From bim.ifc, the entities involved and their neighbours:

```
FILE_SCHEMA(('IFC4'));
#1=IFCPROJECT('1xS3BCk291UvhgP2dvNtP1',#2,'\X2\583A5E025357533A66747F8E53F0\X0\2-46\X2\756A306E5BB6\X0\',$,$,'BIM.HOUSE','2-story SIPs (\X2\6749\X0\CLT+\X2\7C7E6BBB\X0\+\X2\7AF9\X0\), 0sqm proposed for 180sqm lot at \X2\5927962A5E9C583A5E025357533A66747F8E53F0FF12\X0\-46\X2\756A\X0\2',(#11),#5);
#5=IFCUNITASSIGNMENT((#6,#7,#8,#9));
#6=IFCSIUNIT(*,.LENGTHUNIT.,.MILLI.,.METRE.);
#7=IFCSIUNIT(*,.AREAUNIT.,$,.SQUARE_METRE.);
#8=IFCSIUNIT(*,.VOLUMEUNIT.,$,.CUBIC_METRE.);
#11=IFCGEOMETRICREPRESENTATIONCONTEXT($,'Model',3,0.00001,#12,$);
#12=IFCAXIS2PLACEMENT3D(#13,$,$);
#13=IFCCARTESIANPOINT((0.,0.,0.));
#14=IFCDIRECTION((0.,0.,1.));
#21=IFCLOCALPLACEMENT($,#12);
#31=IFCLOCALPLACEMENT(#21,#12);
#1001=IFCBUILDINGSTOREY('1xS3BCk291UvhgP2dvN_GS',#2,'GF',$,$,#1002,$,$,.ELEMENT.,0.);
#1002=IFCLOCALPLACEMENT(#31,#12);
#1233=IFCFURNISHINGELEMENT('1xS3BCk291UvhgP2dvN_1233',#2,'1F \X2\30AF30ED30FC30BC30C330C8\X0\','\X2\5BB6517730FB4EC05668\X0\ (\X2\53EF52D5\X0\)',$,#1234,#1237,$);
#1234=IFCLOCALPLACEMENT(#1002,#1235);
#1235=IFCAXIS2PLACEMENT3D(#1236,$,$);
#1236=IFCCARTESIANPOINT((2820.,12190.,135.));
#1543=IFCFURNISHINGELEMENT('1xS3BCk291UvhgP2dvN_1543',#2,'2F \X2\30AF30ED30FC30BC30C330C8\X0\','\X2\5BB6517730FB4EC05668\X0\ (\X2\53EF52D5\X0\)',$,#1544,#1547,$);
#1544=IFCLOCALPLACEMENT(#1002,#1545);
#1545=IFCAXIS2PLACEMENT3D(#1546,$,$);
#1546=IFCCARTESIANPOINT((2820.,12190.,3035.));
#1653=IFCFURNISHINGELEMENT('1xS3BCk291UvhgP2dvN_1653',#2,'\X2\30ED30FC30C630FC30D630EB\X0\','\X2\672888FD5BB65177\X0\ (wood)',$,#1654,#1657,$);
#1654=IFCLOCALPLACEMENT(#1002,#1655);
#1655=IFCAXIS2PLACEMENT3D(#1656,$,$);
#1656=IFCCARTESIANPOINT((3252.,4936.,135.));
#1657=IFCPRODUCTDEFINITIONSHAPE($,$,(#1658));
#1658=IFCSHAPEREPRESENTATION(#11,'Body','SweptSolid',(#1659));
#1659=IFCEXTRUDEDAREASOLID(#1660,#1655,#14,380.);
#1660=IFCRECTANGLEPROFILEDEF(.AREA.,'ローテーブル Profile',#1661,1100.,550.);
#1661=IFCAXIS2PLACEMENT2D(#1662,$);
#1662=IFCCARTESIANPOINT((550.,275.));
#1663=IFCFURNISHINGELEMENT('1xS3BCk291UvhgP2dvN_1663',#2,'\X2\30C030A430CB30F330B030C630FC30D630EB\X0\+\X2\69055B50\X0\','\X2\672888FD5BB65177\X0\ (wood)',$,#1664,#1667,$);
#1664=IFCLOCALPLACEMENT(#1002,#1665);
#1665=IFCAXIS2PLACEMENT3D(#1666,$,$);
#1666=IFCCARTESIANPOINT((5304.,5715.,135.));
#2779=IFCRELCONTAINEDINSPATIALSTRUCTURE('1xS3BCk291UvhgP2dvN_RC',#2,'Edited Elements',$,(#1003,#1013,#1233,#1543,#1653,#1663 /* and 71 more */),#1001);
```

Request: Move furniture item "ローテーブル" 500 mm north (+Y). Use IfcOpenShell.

```python
import ifcopenshell
import ifcopenshell.api.geometry
import ifcopenshell.util.placement

model = ifcopenshell.open("bim.ifc")

item = model.by_guid("1xS3BCk291UvhgP2dvN_1653")
matrix = ifcopenshell.util.placement.get_local_placement(item.ObjectPlacement)
matrix[1, 3] += 500.0
ifcopenshell.api.geometry.edit_object_placement(model, product=item, matrix=matrix, is_si=False)

print(ifcopenshell.util.placement.get_local_placement(item.ObjectPlacement).round(3) + 0.0)

model.write("bim_v2.ifc")
```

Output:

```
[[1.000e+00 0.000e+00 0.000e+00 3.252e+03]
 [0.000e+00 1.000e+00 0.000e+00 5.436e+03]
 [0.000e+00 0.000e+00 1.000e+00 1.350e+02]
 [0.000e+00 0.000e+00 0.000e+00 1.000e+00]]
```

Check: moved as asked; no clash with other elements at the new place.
